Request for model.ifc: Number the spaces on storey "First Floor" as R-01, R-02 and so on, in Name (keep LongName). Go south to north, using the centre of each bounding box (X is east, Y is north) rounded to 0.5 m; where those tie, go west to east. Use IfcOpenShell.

First a look at what the model holds.

```python
import ifcopenshell
import ifcopenshell.util.element
import ifcopenshell.util.placement

model = ifcopenshell.open("model.ifc")
print(model.schema)
storey = next(s for s in model.by_type("IfcBuildingStorey") if s.Name == "First Floor")
spaces = [e for e in ifcopenshell.util.element.get_decomposition(storey) if e.is_a("IfcSpace")]
for e in sorted(spaces, key=lambda e: e.id()):
    origin = ifcopenshell.util.placement.get_local_placement(e.ObjectPlacement)[:3, 3]
    print(e.id(), e.Name, e.LongName, origin.round(2) + 0.0, sep=" | ")
```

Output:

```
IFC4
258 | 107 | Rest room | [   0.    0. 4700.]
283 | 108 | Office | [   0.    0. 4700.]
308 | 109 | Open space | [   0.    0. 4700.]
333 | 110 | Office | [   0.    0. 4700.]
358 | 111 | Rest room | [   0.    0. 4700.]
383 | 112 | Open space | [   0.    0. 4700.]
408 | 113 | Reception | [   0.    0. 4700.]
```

```python
import ifcopenshell
import ifcopenshell.geom
import ifcopenshell.util.element
import ifcopenshell.util.shape

model = ifcopenshell.open("model.ifc")
settings = ifcopenshell.geom.settings()
settings.set("use-world-coords", True)


def centre(element):
    shape = ifcopenshell.geom.create_shape(settings, element)
    return ifcopenshell.util.shape.get_bbox_centroid(shape.geometry)


storey = next(s for s in model.by_type("IfcBuildingStorey") if s.Name == "First Floor")
spaces = [e for e in ifcopenshell.util.element.get_decomposition(storey) if e.is_a("IfcSpace")]

# Insertion points can sit at a corner or the storey origin, so sort by the geometry (in metres).
centres = {e: centre(e) for e in spaces}
spaces.sort(key=lambda e: (round(centres[e][1] / 0.5), centres[e][0]))

for i, e in enumerate(spaces, start=1):
    number = f"R-{i:02d}"
    e.Name = number
    print(e.id(), number)

model.write("model-out.ifc")
```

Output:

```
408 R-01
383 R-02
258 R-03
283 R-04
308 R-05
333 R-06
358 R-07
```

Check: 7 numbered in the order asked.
